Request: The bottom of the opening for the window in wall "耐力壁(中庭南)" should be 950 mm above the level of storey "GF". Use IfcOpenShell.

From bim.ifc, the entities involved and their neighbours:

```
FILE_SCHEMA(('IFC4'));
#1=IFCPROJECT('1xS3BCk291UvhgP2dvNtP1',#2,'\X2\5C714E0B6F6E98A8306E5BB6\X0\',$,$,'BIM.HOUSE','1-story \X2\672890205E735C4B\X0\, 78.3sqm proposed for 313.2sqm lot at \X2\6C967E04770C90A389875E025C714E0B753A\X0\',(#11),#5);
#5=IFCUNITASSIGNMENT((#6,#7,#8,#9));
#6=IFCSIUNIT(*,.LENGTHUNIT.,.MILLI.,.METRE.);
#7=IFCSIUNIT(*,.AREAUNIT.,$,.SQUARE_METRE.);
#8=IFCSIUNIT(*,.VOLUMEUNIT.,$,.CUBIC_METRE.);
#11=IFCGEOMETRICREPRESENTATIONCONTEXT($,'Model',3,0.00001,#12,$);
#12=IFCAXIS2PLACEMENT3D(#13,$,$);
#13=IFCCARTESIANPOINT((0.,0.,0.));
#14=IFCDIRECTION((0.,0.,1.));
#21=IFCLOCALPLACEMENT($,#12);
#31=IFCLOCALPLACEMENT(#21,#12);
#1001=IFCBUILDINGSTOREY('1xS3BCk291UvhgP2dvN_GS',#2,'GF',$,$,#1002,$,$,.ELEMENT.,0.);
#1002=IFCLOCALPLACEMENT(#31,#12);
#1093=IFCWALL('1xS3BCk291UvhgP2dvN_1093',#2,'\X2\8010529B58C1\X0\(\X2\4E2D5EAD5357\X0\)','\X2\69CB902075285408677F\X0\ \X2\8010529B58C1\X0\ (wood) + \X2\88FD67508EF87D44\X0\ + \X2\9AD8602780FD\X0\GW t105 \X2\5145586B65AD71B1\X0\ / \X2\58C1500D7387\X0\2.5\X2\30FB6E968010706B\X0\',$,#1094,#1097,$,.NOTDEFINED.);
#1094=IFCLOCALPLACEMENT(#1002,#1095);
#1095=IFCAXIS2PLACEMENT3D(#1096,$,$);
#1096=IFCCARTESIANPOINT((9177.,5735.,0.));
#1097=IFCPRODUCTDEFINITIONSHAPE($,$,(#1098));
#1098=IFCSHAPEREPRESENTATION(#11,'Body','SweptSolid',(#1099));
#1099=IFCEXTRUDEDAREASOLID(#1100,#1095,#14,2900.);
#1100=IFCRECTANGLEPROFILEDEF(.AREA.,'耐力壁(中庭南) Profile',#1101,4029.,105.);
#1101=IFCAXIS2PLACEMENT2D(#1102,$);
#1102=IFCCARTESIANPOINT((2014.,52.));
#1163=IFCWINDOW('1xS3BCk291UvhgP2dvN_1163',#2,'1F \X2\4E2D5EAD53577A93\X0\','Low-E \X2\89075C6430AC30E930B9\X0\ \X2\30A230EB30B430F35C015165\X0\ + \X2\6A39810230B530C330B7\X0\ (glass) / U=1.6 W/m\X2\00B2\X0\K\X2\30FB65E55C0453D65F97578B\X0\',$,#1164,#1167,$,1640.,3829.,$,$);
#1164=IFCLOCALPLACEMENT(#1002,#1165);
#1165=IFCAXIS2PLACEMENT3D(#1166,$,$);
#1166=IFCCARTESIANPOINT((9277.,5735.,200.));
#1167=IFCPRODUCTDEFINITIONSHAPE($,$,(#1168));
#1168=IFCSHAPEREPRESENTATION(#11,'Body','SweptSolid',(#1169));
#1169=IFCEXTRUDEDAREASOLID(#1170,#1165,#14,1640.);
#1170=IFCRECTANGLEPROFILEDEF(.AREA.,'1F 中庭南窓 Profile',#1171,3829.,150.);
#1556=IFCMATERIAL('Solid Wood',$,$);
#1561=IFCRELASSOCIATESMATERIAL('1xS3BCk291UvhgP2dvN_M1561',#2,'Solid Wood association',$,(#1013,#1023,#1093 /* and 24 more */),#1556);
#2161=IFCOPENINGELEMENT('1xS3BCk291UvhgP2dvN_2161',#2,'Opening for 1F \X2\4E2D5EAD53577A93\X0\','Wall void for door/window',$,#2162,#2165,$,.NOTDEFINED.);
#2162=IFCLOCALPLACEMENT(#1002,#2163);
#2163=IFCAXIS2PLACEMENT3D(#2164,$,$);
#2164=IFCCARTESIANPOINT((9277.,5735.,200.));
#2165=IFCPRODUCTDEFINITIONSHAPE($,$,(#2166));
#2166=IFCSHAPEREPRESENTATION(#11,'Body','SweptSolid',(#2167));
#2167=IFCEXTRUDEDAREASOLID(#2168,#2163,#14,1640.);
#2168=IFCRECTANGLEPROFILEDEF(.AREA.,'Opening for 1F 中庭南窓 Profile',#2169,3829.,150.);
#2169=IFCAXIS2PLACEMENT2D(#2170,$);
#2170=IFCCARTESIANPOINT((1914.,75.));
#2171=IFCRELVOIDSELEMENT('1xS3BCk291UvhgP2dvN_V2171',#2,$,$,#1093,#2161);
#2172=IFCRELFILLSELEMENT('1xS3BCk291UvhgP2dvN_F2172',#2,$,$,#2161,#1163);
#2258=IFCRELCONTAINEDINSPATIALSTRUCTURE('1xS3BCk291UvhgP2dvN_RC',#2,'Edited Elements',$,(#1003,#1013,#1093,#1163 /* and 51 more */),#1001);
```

```python
import numpy as np
import ifcopenshell
import ifcopenshell.api.geometry
import ifcopenshell.geom
import ifcopenshell.util.element
import ifcopenshell.util.placement
import ifcopenshell.util.shape
import ifcopenshell.util.unit

model = ifcopenshell.open("bim.ifc")
unit_scale = ifcopenshell.util.unit.calculate_unit_scale(model)

window = model.by_id(1163)
opening = window.FillsVoids[0].RelatingOpeningElement
storey = ifcopenshell.util.element.get_container(window, ifc_class="IfcBuildingStorey")
level = ifcopenshell.util.placement.get_local_placement(storey.ObjectPlacement)[2, 3]

# The opening's origin need not be at the sill, so measure its lowest point.
shape = ifcopenshell.geom.create_shape(ifcopenshell.geom.settings(), opening)
bottom = ifcopenshell.util.shape.get_shape_bottom_elevation(shape, shape.geometry) / unit_scale
dz = level + 950.0 - bottom

shift = np.array([0.0, 0.0, dz])
# The window is not placed relative to its opening, so move both.
for product in (opening, window):
    matrix = ifcopenshell.util.placement.get_local_placement(product.ObjectPlacement)
    matrix[:3, 3] += shift
    ifcopenshell.api.geometry.edit_object_placement(model, product=product, matrix=matrix, is_si=False)

print(f"moved by {dz * unit_scale:+.3f} m")

model.write("bim_rev.ifc")
```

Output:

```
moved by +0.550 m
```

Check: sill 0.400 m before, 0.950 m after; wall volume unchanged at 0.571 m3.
